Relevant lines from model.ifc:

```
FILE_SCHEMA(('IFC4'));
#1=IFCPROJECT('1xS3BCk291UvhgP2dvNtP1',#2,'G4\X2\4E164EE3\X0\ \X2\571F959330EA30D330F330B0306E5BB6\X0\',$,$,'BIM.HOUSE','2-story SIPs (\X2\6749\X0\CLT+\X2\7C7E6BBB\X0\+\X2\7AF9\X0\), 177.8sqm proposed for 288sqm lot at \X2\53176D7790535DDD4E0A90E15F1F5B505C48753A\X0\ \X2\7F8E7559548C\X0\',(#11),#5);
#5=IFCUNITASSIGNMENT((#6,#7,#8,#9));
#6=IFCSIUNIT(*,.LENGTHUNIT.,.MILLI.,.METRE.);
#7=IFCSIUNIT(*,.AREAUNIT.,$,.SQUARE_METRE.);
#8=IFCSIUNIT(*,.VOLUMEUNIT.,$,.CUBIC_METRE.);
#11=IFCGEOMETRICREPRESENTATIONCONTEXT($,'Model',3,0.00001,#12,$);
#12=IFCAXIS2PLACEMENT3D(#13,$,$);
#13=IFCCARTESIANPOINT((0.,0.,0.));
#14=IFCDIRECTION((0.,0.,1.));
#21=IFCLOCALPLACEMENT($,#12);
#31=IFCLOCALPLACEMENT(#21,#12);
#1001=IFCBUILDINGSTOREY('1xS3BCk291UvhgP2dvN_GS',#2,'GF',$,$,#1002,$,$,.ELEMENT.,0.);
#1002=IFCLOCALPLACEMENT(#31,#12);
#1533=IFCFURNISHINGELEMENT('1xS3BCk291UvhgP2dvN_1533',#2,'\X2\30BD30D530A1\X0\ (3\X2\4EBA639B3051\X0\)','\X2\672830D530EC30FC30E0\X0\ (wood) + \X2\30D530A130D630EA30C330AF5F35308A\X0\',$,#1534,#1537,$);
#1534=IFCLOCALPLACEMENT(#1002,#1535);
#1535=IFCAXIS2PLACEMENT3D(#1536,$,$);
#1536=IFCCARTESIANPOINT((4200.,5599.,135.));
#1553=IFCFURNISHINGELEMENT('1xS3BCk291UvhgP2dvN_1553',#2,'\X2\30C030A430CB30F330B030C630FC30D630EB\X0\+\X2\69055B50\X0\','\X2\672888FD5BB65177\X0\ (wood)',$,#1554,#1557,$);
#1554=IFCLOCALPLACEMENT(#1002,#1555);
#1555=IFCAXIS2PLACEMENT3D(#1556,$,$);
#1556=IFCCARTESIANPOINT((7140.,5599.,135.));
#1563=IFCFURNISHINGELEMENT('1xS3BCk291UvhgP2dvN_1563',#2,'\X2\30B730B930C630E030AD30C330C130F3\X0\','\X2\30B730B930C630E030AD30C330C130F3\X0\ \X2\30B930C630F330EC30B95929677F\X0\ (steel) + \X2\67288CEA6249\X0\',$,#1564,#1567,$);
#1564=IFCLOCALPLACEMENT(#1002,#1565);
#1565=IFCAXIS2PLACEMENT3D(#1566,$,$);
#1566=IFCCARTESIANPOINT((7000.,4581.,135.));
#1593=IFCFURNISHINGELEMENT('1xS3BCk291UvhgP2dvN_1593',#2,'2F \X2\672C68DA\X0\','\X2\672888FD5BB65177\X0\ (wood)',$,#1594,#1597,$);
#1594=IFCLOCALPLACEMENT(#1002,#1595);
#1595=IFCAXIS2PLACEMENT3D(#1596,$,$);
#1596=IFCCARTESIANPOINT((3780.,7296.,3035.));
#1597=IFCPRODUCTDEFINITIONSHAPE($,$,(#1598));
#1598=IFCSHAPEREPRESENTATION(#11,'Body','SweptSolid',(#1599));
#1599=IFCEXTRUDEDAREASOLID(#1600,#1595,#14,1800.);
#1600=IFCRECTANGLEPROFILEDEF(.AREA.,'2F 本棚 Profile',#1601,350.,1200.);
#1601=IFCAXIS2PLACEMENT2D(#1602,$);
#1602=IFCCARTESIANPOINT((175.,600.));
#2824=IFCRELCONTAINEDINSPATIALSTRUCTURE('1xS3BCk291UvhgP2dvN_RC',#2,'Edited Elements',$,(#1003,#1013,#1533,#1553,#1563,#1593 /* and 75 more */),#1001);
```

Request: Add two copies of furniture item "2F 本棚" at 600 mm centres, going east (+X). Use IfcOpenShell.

```python
import numpy as np
import ifcopenshell
import ifcopenshell.api.geometry
import ifcopenshell.api.root
import ifcopenshell.util.element
import ifcopenshell.util.placement

model = ifcopenshell.open("model.ifc")


def reuse_history(source, copy):
    """copy_class also copies each property set's owner history, people and application; keep the originals."""
    for rel in copy.IsDefinedBy:
        if rel.is_a("IfcRelDefinesByProperties") and (history := rel.RelatingPropertyDefinition.OwnerHistory):
            rel.RelatingPropertyDefinition.OwnerHistory = source.OwnerHistory
            ifcopenshell.util.element.remove_deep2(model, history)


source = model.by_guid("1xS3BCk291UvhgP2dvN_1593")
base = ifcopenshell.util.placement.get_local_placement(source.ObjectPlacement)
step = np.array([1.0, 0.0, 0.0]) * 600.0

for i in range(1, 3):
    copy = ifcopenshell.api.root.copy_class(model, product=source)
    copy.Representation = ifcopenshell.util.element.copy_deep(
        model, source.Representation, exclude=["IfcGeometricRepresentationContext", "IfcRepresentationMap"]
    )
    reuse_history(source, copy)
    matrix = base.copy()
    matrix[:3, 3] += i * step
    print("added at", matrix[:3, 3].round(3) + 0.0)
    ifcopenshell.api.geometry.edit_object_placement(model, product=copy, matrix=matrix, is_si=False)

model.write("model_v2.ifc")
```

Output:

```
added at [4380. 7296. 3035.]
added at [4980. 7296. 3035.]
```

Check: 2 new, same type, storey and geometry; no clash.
